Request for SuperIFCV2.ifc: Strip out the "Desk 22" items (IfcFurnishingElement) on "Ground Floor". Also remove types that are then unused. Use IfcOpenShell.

First a look at what the model holds.

```python
import ifcopenshell
import ifcopenshell.util.element

model = ifcopenshell.open("SuperIFCV2.ifc")
print(model.schema)
storey = next(s for s in model.by_type("IfcBuildingStorey") if s.Name == "Ground Floor")
furniture = [e for e in ifcopenshell.util.element.get_decomposition(storey) if e.is_a("IfcFurnishingElement")]
seen = {}
for e in furniture:
    element_type = ifcopenshell.util.element.get_type(e)
    name = element_type.Name if element_type not in (None, e) else None
    seen[name] = seen.get(name, 0) + 1
for name, count in sorted(seen.items(), key=str):
    print(count, "x", name)
```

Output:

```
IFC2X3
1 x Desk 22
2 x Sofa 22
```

```python
import ifcopenshell
import ifcopenshell.api.root
import ifcopenshell.util.element

model = ifcopenshell.open("SuperIFCV2.ifc")

storey = next(s for s in model.by_type("IfcBuildingStorey") if s.Name == "Ground Floor")
furniture = [e for e in ifcopenshell.util.element.get_decomposition(storey) if e.is_a("IfcFurnishingElement")]
targets = [e for e in furniture if (t := ifcopenshell.util.element.get_type(e)) not in (None, e) and t.Name == "Desk 22"]
types = {ifcopenshell.util.element.get_type(e) for e in targets} - {None, *targets}

for e in targets:
    ifcopenshell.api.root.remove_product(model, product=e)
print(len(targets), "removed")

unused = [t for t in types if not ifcopenshell.util.element.get_types(t)]
for t in unused:
    ifcopenshell.api.root.remove_product(model, product=t)
print(len(unused), "unused types removed")

model.write("SuperIFCV2_updated.ifc")
```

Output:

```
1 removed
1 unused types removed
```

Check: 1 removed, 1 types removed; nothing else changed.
